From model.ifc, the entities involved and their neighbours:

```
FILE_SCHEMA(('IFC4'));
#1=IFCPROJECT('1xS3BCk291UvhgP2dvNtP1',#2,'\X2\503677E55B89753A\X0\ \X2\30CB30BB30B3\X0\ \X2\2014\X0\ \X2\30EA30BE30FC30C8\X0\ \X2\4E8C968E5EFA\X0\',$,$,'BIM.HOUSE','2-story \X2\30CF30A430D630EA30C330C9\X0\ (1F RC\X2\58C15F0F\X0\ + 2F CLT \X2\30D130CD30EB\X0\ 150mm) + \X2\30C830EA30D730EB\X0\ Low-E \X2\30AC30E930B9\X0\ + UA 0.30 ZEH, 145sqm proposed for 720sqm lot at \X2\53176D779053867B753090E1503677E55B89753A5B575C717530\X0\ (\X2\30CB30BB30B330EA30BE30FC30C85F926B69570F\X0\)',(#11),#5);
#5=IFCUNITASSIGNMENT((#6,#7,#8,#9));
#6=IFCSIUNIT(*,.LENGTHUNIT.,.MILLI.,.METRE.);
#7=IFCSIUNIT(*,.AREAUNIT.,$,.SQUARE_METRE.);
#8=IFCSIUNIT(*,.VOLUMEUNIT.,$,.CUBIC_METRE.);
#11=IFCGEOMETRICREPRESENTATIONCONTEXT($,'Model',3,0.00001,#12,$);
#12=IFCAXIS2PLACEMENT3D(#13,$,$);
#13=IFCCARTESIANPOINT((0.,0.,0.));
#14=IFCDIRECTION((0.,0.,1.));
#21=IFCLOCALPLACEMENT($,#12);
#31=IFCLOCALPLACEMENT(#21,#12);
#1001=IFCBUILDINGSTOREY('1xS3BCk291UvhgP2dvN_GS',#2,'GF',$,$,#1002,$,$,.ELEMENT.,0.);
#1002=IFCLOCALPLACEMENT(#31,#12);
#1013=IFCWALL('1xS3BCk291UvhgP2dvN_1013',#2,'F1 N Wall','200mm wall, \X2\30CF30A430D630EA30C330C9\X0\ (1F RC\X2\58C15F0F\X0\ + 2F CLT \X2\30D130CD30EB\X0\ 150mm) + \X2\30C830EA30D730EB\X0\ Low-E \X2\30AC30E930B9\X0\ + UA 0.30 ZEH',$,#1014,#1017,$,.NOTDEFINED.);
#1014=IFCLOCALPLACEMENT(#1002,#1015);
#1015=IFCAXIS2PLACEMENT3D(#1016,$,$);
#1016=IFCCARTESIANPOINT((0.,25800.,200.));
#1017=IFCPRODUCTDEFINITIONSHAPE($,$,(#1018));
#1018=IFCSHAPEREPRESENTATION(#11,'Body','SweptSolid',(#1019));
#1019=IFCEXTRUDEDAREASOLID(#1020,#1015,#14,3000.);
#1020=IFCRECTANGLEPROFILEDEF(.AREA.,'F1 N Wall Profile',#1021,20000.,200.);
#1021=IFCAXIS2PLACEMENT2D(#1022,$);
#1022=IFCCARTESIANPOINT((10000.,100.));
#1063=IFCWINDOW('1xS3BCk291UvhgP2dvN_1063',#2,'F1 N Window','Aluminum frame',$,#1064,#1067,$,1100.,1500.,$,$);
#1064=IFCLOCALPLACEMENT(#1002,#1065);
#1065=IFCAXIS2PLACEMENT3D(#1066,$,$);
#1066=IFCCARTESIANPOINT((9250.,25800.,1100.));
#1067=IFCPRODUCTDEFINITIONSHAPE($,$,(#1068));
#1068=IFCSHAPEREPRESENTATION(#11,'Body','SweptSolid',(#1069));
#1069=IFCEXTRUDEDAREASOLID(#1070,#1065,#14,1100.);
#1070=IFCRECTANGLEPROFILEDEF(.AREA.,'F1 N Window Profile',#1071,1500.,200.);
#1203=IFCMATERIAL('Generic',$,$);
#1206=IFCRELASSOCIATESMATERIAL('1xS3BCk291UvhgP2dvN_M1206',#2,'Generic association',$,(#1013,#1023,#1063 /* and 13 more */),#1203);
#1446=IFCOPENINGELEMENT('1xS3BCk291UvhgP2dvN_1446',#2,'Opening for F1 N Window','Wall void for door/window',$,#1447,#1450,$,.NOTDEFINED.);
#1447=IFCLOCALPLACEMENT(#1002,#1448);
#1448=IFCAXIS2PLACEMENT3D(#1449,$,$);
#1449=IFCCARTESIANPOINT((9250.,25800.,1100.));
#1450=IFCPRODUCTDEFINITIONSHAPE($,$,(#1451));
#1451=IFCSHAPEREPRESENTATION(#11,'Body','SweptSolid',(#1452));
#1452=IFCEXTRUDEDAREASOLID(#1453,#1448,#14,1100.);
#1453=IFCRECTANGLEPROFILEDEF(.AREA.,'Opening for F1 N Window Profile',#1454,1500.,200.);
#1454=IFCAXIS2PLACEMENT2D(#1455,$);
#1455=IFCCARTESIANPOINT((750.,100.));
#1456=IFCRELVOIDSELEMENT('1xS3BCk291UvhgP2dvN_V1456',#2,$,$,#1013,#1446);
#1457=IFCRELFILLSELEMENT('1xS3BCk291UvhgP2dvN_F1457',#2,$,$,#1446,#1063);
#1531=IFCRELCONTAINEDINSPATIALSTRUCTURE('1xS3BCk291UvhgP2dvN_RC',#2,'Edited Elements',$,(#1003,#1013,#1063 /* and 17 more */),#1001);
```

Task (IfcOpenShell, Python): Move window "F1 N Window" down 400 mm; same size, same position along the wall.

```python
import numpy as np
import ifcopenshell
import ifcopenshell.api.geometry
import ifcopenshell.util.placement
import ifcopenshell.util.unit

model = ifcopenshell.open("model.ifc")
unit_scale = ifcopenshell.util.unit.calculate_unit_scale(model)

window = model.by_guid("1xS3BCk291UvhgP2dvN_1063")
opening = window.FillsVoids[0].RelatingOpeningElement
dz = -0.4 / unit_scale

shift = np.array([0.0, 0.0, dz])
# The window is not placed relative to its opening, so move both.
for product in (opening, window):
    matrix = ifcopenshell.util.placement.get_local_placement(product.ObjectPlacement)
    matrix[:3, 3] += shift
    ifcopenshell.api.geometry.edit_object_placement(model, product=product, matrix=matrix, is_si=False)

print(f"moved by {dz * unit_scale:+.3f} m")

model.write("model-out.ifc")
```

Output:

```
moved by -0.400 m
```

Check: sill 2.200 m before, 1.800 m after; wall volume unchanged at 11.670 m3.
